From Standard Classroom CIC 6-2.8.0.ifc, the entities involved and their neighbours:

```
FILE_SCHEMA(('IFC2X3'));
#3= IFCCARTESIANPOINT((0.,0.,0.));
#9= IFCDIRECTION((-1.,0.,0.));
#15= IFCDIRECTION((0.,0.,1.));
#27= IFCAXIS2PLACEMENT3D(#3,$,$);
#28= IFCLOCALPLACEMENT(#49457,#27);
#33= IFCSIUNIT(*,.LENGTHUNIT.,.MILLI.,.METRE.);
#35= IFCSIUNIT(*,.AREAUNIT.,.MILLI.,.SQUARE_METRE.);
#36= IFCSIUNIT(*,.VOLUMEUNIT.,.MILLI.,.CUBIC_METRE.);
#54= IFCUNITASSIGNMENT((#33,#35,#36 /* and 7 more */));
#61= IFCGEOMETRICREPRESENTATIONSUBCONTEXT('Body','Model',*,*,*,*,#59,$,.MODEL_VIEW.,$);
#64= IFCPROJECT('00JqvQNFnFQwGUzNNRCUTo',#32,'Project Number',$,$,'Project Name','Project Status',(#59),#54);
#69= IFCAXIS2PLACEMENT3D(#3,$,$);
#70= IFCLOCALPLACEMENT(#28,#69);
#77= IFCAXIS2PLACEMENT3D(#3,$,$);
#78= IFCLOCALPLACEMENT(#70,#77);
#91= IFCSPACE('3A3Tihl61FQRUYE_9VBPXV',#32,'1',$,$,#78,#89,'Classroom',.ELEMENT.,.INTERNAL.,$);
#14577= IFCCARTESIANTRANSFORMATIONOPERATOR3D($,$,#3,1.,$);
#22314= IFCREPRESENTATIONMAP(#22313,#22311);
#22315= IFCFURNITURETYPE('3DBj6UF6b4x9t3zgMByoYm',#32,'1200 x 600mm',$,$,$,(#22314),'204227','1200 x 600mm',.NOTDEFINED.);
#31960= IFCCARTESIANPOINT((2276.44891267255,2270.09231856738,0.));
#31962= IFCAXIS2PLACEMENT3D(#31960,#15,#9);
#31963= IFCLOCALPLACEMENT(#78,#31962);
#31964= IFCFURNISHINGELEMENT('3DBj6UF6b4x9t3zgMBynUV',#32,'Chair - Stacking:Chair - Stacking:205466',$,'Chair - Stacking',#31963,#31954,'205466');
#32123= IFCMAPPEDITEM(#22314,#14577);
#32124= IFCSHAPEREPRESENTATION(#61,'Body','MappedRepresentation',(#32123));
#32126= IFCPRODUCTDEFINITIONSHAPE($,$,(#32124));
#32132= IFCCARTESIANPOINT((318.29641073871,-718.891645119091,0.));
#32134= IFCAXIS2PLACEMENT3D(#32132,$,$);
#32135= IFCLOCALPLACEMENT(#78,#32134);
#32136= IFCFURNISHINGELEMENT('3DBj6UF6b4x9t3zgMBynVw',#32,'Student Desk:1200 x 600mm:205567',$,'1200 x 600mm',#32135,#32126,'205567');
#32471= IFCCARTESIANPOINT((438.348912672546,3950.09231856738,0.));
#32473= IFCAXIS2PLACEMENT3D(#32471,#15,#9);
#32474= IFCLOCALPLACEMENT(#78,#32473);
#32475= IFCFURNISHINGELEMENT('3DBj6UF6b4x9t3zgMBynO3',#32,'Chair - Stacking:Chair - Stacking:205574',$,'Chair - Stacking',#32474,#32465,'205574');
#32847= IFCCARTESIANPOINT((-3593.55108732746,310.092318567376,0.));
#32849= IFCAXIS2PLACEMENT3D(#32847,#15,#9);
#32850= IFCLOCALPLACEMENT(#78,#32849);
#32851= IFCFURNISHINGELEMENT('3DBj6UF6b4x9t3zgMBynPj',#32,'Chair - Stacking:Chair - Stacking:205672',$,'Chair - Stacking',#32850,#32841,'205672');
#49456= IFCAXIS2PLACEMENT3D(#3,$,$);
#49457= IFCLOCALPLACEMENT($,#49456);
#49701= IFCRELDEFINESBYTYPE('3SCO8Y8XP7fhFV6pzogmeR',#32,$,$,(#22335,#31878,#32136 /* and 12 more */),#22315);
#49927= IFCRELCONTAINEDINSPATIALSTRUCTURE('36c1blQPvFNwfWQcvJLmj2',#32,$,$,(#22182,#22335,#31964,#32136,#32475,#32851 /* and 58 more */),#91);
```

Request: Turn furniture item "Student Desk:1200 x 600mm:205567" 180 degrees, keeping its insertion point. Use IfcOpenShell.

```python
import ifcopenshell
import ifcopenshell.api.geometry
import ifcopenshell.util.placement

model = ifcopenshell.open("Standard Classroom CIC 6-2.8.0.ifc")

item = model.by_guid("3DBj6UF6b4x9t3zgMBynVw")
matrix = ifcopenshell.util.placement.get_local_placement(item.ObjectPlacement)
matrix = matrix @ ifcopenshell.util.placement.rotation(180, "Z")
ifcopenshell.api.geometry.edit_object_placement(model, product=item, matrix=matrix, is_si=False)

print(ifcopenshell.util.placement.get_local_placement(item.ObjectPlacement).round(3) + 0.0)

model.write("Standard Classroom CIC 6-2.8.0_rev.ifc")
```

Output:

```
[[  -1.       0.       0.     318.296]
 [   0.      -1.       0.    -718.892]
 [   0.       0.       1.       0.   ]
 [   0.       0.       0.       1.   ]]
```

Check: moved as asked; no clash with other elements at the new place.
